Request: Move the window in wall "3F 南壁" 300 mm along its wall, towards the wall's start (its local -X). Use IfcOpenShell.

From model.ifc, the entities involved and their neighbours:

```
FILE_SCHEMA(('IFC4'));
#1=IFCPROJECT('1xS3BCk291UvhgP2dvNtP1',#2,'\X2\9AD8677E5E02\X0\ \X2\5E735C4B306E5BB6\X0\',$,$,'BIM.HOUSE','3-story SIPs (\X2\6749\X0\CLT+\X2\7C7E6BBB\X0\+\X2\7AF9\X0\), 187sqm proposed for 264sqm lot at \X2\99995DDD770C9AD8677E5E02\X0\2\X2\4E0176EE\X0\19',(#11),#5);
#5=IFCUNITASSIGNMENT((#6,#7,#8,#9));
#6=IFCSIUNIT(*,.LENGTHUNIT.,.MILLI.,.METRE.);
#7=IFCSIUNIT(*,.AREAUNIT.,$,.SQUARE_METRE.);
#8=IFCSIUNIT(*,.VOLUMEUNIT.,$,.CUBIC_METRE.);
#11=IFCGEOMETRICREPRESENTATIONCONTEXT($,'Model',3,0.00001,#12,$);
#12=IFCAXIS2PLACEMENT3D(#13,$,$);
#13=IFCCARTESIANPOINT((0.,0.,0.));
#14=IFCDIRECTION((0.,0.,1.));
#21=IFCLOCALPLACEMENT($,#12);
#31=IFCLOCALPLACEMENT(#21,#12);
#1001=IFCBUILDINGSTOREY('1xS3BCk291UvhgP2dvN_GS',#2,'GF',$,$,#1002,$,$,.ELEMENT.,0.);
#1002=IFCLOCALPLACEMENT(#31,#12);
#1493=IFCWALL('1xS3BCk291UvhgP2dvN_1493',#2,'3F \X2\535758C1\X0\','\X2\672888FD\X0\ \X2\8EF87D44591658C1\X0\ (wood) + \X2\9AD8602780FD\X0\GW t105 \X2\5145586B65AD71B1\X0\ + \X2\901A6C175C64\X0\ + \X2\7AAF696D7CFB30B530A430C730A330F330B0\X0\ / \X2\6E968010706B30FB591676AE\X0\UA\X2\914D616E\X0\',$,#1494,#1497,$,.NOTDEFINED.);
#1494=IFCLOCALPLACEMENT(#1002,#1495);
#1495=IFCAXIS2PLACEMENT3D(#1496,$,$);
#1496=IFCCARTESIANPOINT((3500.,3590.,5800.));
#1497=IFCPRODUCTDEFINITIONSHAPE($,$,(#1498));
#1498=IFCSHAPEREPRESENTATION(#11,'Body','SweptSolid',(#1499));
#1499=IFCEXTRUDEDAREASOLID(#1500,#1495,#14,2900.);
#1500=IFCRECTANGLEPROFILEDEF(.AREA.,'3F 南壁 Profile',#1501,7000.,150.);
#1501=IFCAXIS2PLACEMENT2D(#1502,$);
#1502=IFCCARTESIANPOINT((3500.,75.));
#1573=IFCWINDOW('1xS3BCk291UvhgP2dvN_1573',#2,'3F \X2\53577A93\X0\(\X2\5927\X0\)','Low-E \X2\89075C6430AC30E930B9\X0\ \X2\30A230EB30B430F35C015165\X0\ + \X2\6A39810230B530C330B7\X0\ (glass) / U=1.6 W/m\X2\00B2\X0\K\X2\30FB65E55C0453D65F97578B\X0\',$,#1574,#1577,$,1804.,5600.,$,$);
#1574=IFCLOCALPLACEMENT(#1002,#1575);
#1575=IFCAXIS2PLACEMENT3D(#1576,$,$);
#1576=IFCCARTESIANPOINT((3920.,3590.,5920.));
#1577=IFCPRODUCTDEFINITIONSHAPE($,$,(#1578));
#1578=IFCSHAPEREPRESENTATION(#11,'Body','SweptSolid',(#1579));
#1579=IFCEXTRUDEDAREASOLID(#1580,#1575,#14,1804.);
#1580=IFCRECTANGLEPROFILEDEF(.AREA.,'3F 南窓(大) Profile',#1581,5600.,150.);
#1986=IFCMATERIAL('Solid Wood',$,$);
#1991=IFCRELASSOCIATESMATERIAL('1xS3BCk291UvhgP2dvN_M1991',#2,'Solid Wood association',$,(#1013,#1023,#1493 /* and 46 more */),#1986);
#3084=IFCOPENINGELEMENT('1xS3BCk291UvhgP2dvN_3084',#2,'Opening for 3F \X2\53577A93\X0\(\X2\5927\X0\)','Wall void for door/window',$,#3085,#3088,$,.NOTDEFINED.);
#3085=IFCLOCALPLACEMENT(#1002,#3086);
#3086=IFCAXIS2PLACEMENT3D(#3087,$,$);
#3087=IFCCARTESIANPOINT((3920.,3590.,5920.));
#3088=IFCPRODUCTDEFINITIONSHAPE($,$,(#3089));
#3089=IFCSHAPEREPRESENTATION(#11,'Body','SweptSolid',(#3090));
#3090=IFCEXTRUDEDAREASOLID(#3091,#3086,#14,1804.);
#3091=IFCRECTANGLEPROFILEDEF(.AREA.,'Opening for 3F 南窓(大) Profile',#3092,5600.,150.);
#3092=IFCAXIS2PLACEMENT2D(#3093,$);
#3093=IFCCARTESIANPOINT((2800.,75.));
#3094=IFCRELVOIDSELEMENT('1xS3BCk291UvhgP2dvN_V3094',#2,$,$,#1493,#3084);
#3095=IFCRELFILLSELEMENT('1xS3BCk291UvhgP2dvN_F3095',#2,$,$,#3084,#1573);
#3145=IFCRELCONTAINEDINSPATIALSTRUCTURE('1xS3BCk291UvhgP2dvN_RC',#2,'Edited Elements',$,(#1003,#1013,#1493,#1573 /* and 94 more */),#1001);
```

```python
import ifcopenshell
import ifcopenshell.api.geometry
import ifcopenshell.util.placement
import ifcopenshell.util.unit

model = ifcopenshell.open("model.ifc")
unit_scale = ifcopenshell.util.unit.calculate_unit_scale(model)

window = model.by_guid("1xS3BCk291UvhgP2dvN_1573")
opening = window.FillsVoids[0].RelatingOpeningElement
wall = opening.VoidsElements[0].RelatingBuildingElement

wall_matrix = ifcopenshell.util.placement.get_local_placement(wall.ObjectPlacement)
shift = wall_matrix[:3, 0] * -0.3 / unit_scale
before = ifcopenshell.util.placement.get_local_placement(window.ObjectPlacement)[:3, 3].copy()

# The window is not placed relative to its opening, so move both.
for product in (opening, window):
    matrix = ifcopenshell.util.placement.get_local_placement(product.ObjectPlacement)
    matrix[:3, 3] += shift
    ifcopenshell.api.geometry.edit_object_placement(model, product=product, matrix=matrix, is_si=False)

after = ifcopenshell.util.placement.get_local_placement(window.ObjectPlacement)[:3, 3]
print("window moved by", (after - before).round(3) + 0.0)

model.write("model_updated.ifc")
```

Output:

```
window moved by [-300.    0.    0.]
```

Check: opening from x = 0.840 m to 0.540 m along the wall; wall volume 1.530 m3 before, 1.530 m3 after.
